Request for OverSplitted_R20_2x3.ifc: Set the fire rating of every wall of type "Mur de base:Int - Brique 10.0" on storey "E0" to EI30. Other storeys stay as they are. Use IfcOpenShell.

First a look at what the model holds.

```python
import ifcopenshell
import ifcopenshell.util.element

model = ifcopenshell.open("OverSplitted_R20_2x3.ifc")
print(model.schema)
storey = next(s for s in model.by_type("IfcBuildingStorey") if s.Name == "E0")
walls = [e for e in ifcopenshell.util.element.get_decomposition(storey) if e.is_a("IfcWall")]
seen = {}
for e in walls:
    element_type = ifcopenshell.util.element.get_type(e)
    key = (element_type.Name if element_type != e and element_type else None, ifcopenshell.util.element.get_pset(e, "Pset_WallCommon", "FireRating"))
    seen[key] = seen.get(key, 0) + 1
for (name, value), count in sorted(seen.items(), key=str):
    print(count, "x", name, "|", value)
```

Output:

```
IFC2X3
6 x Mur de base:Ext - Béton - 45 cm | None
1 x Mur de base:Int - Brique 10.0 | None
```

```python
import ifcopenshell
import ifcopenshell.api.pset
import ifcopenshell.util.element

model = ifcopenshell.open("OverSplitted_R20_2x3.ifc")

storey = next(s for s in model.by_type("IfcBuildingStorey") if s.Name == "E0")
walls = [e for e in ifcopenshell.util.element.get_decomposition(storey) if e.is_a("IfcWall")]

count = 0
for e in walls:
    element_type = ifcopenshell.util.element.get_type(e)
    if element_type in (None, e) or element_type.Name != "Mur de base:Int - Brique 10.0":
        continue
    # add_pset returns the element's existing set when there is one.
    pset = ifcopenshell.api.pset.add_pset(model, product=e, name="Pset_WallCommon")
    ifcopenshell.api.pset.edit_pset(model, pset=pset, properties={"FireRating": "EI30"})
    count += 1

print(count, "walls updated")

model.write("OverSplitted_R20_2x3-out.ifc")
```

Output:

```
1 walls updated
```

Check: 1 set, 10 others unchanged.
